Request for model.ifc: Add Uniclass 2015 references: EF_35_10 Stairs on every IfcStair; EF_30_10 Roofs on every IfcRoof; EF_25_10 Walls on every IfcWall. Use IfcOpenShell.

First a look at what the model holds.

```python
import ifcopenshell

model = ifcopenshell.open("model.ifc")
print(model.schema)
print("classifications:", [c.Name for c in model.by_type("IfcClassification")])
for ifc_class in ("IfcDoor", "IfcRoof", "IfcStair", "IfcWall", "IfcWindow"):
    print(ifc_class, len(model.by_type(ifc_class)))
```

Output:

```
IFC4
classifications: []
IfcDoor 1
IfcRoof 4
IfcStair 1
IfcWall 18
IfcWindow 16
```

```python
import ifcopenshell
import ifcopenshell.api.classification

model = ifcopenshell.open("model.ifc")

system = ifcopenshell.api.classification.add_classification(model, classification="Uniclass 2015")

codes = {
    "IfcStair": ("EF_35_10", "Stairs"),
    "IfcRoof": ("EF_30_10", "Roofs"),
    "IfcWall": ("EF_25_10", "Walls"),
}
for ifc_class, (code, name) in codes.items():
    products = model.by_type(ifc_class)
    ifcopenshell.api.classification.add_reference(
        model, products=products, classification=system, identification=code, name=name
    )
    print(code, len(products))

model.write("model_edited.ifc")
```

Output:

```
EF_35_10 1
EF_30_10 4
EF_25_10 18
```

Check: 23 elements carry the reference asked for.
